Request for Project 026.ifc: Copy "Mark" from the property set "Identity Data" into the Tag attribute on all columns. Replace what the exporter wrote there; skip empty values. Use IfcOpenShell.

First a look at what the model holds.

```python
import ifcopenshell
import ifcopenshell.util.element

model = ifcopenshell.open("Project 026.ifc")
print(model.schema)
columns = model.by_type("IfcColumn")
print(len(columns), "columns")
for e in columns[:8]:
    source = ifcopenshell.util.element.get_pset(e, "Identity Data", "Mark")
    target = e.Tag
    print(e.id(), repr(source), repr(target), sep=" | ")
```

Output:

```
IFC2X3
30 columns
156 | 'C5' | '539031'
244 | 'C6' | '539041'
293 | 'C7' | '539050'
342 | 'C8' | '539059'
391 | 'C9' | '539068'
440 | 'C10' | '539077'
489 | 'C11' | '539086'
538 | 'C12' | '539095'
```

```python
import ifcopenshell
import ifcopenshell.util.element

model = ifcopenshell.open("Project 026.ifc")

count = 0
for e in model.by_type("IfcColumn"):
    value = ifcopenshell.util.element.get_pset(e, "Identity Data", "Mark")
    current = e.Tag
    if not value or not value.strip() or current == value:
        continue
    e.Tag = value
    count += 1

print(count, "columns updated")

model.write("Project 026_v2.ifc")
```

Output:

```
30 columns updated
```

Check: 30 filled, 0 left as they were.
